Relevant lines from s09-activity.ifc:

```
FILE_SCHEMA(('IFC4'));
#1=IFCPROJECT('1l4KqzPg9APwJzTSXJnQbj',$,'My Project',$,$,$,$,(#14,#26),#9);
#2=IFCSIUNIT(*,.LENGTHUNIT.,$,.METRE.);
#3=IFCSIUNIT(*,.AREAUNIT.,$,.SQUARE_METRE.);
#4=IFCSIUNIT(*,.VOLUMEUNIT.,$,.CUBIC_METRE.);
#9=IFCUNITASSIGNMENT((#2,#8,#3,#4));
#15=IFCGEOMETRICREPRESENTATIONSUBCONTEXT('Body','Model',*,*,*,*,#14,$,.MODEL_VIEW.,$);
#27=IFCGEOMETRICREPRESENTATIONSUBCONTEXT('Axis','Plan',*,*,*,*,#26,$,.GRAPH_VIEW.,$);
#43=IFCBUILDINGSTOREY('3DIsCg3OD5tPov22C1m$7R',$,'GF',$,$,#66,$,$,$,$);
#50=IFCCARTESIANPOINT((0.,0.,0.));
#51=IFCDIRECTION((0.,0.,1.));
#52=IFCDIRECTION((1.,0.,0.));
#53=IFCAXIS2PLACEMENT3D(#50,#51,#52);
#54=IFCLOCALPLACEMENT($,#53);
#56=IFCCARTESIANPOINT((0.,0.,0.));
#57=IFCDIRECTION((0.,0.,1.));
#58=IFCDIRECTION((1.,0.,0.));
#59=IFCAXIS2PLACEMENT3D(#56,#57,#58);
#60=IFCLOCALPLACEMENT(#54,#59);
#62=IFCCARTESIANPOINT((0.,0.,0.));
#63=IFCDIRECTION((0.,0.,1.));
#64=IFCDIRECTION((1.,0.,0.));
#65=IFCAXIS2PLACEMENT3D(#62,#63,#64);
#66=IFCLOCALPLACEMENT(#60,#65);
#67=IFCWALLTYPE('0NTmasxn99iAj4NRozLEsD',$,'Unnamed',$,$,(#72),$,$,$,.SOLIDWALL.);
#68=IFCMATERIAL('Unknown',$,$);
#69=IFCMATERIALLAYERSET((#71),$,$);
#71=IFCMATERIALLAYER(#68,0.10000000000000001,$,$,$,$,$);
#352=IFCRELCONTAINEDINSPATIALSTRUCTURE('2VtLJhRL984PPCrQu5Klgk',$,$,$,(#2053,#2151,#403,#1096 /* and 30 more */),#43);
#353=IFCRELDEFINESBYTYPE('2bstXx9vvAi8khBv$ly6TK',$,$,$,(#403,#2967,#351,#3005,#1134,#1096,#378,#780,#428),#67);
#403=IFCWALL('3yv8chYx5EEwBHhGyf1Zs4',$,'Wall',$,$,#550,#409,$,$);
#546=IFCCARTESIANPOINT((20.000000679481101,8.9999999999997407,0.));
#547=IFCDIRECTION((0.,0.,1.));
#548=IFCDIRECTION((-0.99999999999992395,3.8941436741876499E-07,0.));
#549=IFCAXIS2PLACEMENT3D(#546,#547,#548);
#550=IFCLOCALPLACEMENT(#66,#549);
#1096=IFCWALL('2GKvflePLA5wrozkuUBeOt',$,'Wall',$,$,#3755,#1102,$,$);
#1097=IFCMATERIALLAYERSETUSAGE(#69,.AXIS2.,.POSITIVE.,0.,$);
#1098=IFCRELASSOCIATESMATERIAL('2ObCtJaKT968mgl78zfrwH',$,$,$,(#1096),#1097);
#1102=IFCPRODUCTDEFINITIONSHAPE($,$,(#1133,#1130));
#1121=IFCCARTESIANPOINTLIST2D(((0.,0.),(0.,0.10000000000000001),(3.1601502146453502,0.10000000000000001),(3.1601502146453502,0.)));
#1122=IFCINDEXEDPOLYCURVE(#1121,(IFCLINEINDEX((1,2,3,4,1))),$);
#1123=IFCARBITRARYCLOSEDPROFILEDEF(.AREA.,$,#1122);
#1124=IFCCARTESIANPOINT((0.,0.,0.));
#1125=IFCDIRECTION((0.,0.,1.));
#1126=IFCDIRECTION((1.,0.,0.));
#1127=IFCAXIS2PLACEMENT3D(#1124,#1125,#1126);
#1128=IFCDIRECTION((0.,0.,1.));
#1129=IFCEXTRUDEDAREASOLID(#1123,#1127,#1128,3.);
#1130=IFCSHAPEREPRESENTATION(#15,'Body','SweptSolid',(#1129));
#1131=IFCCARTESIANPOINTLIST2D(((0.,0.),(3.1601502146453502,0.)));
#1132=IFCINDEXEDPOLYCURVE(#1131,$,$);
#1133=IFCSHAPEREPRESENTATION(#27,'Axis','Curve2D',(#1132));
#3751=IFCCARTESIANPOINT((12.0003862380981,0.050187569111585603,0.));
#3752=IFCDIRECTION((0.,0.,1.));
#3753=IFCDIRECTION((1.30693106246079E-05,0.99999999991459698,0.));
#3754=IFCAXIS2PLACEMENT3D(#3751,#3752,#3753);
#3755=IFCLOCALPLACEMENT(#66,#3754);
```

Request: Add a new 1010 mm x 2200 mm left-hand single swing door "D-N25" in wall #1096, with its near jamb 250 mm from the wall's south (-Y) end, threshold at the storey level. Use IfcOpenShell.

```python
import numpy as np
import ifcopenshell
import ifcopenshell.api.feature
import ifcopenshell.api.geometry
import ifcopenshell.api.root
import ifcopenshell.api.spatial
import ifcopenshell.geom
import ifcopenshell.util.element
import ifcopenshell.util.placement
import ifcopenshell.util.representation
import ifcopenshell.util.shape
import ifcopenshell.util.unit

model = ifcopenshell.open("s09-activity.ifc")
unit_scale = ifcopenshell.util.unit.calculate_unit_scale(model)
settings = ifcopenshell.geom.settings()


def volume(element):
    """Net volume in cubic metres, openings subtracted."""
    shape = ifcopenshell.geom.create_shape(settings, element)
    return ifcopenshell.util.shape.get_volume(shape.geometry)


wall = model.by_guid("2GKvflePLA5wrozkuUBeOt")
storey = ifcopenshell.util.element.get_container(wall, ifc_class="IfcBuildingStorey")
context = ifcopenshell.util.representation.get_context(model, "Model", "Body", "MODEL_VIEW")
before = volume(wall)

width, height, from_end, sill = 1.01, 2.2, 0.25, 0.0  # metres

# The wall runs along its own X axis, and the end named is its -X end.
wall_shape = ifcopenshell.geom.create_shape(settings, wall)
x, y, z = ifcopenshell.util.shape.get_vertices(wall_shape.geometry).T
start = x.min() + from_end
face, thickness = float(y.min()), float(y.max() - y.min())
wall_matrix = ifcopenshell.util.placement.get_local_placement(wall.ObjectPlacement)
level = ifcopenshell.util.placement.get_local_placement(storey.ObjectPlacement)[2, 3]


def in_wall(x, y):
    """Placement at x, y metres in the wall's axes, at sill height."""
    matrix = wall_matrix.copy()
    matrix[:, 3] = wall_matrix @ np.array([x / unit_scale, y / unit_scale, 0.0, 1.0])
    matrix[2, 3] = level + sill / unit_scale
    return matrix


# Opening: a box that overshoots both wall faces by 50 mm.
opening = ifcopenshell.api.root.create_entity(model, ifc_class="IfcOpeningElement", predefined_type="OPENING")
box = ifcopenshell.api.geometry.add_wall_representation(
    model, context=context, length=width, height=height, thickness=thickness + 0.1
)
ifcopenshell.api.geometry.assign_representation(model, product=opening, representation=box)
ifcopenshell.api.geometry.edit_object_placement(model, product=opening, matrix=in_wall(start, face - 0.05), is_si=False)
ifcopenshell.api.feature.add_feature(model, feature=opening, element=wall)

door = ifcopenshell.api.root.create_entity(model, ifc_class="IfcDoor", name="D-N25", predefined_type="DOOR")
door.OverallWidth, door.OverallHeight = width / unit_scale, height / unit_scale
door.OperationType = "SINGLE_SWING_LEFT"
body = ifcopenshell.api.geometry.add_door_representation(
    model,
    context=context,
    overall_width=door.OverallWidth,
    overall_height=door.OverallHeight,
    operation_type="SINGLE_SWING_LEFT",
    lining_properties={"LiningDepth": thickness / unit_scale, "ThresholdDepth": thickness / unit_scale},
)
ifcopenshell.api.geometry.assign_representation(model, product=door, representation=body)
ifcopenshell.api.spatial.assign_container(model, products=[door], relating_structure=storey)
ifcopenshell.api.feature.add_filling(model, opening=opening, element=door)

# The lining spans the wall, so the door starts at the wall face.
ifcopenshell.api.geometry.edit_object_placement(model, product=door, matrix=in_wall(start, face), is_si=False)

after = volume(wall)

print(f"wall volume {before:.3f} -> {after:.3f} m3")

model.write("s09-activity_updated.ifc")
```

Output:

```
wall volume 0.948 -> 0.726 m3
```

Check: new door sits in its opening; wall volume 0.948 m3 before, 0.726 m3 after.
